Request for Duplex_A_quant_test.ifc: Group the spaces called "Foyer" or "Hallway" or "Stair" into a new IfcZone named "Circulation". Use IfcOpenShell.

First a look at what the model holds.

```python
import ifcopenshell

model = ifcopenshell.open("Duplex_A_quant_test.ifc")
print(model.schema)
seen = {}
for space in model.by_type("IfcSpace"):
    seen[space.LongName] = seen.get(space.LongName, 0) + 1
for name, count in sorted(seen.items(), key=str):
    print(count, "x", name)
print("zones:", [z.Name for z in model.by_type("IfcZone")][:20])
```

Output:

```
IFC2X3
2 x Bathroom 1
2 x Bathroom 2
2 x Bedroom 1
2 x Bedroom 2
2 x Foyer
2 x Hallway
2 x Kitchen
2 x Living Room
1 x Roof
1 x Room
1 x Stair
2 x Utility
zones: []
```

```python
import ifcopenshell
import ifcopenshell.api.group
import ifcopenshell.api.root

model = ifcopenshell.open("Duplex_A_quant_test.ifc")

names = {"Foyer", "Hallway", "Stair"}
spaces = [s for s in model.by_type("IfcSpace") if s.LongName in names]

zone = ifcopenshell.api.root.create_entity(model, ifc_class="IfcZone", name="Circulation")
ifcopenshell.api.group.assign_group(model, products=spaces, group=zone)
print(len(spaces), "spaces in", zone.Name)

model.write("Duplex_A_quant_test_edited.ifc")
```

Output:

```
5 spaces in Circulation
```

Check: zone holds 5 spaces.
